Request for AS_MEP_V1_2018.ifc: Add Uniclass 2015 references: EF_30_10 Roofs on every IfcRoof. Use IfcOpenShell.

First a look at what the model holds.

```python
import ifcopenshell

model = ifcopenshell.open("AS_MEP_V1_2018.ifc")
print(model.schema)
print("classifications:", [c.Name for c in model.by_type("IfcClassification")])
for ifc_class in ("IfcDoor", "IfcRoof", "IfcStair", "IfcWall", "IfcWindow"):
    print(ifc_class, len(model.by_type(ifc_class)))
```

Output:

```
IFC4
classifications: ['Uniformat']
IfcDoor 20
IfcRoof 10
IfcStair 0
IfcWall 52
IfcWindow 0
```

```python
import ifcopenshell
import ifcopenshell.api.classification

model = ifcopenshell.open("AS_MEP_V1_2018.ifc")

system = ifcopenshell.api.classification.add_classification(model, classification="Uniclass 2015")

codes = {
    "IfcRoof": ("EF_30_10", "Roofs"),
}
for ifc_class, (code, name) in codes.items():
    products = model.by_type(ifc_class)
    ifcopenshell.api.classification.add_reference(
        model, products=products, classification=system, identification=code, name=name
    )
    print(code, len(products))

model.write("AS_MEP_V1_2018_v2.ifc")
```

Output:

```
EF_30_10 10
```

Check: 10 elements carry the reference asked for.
